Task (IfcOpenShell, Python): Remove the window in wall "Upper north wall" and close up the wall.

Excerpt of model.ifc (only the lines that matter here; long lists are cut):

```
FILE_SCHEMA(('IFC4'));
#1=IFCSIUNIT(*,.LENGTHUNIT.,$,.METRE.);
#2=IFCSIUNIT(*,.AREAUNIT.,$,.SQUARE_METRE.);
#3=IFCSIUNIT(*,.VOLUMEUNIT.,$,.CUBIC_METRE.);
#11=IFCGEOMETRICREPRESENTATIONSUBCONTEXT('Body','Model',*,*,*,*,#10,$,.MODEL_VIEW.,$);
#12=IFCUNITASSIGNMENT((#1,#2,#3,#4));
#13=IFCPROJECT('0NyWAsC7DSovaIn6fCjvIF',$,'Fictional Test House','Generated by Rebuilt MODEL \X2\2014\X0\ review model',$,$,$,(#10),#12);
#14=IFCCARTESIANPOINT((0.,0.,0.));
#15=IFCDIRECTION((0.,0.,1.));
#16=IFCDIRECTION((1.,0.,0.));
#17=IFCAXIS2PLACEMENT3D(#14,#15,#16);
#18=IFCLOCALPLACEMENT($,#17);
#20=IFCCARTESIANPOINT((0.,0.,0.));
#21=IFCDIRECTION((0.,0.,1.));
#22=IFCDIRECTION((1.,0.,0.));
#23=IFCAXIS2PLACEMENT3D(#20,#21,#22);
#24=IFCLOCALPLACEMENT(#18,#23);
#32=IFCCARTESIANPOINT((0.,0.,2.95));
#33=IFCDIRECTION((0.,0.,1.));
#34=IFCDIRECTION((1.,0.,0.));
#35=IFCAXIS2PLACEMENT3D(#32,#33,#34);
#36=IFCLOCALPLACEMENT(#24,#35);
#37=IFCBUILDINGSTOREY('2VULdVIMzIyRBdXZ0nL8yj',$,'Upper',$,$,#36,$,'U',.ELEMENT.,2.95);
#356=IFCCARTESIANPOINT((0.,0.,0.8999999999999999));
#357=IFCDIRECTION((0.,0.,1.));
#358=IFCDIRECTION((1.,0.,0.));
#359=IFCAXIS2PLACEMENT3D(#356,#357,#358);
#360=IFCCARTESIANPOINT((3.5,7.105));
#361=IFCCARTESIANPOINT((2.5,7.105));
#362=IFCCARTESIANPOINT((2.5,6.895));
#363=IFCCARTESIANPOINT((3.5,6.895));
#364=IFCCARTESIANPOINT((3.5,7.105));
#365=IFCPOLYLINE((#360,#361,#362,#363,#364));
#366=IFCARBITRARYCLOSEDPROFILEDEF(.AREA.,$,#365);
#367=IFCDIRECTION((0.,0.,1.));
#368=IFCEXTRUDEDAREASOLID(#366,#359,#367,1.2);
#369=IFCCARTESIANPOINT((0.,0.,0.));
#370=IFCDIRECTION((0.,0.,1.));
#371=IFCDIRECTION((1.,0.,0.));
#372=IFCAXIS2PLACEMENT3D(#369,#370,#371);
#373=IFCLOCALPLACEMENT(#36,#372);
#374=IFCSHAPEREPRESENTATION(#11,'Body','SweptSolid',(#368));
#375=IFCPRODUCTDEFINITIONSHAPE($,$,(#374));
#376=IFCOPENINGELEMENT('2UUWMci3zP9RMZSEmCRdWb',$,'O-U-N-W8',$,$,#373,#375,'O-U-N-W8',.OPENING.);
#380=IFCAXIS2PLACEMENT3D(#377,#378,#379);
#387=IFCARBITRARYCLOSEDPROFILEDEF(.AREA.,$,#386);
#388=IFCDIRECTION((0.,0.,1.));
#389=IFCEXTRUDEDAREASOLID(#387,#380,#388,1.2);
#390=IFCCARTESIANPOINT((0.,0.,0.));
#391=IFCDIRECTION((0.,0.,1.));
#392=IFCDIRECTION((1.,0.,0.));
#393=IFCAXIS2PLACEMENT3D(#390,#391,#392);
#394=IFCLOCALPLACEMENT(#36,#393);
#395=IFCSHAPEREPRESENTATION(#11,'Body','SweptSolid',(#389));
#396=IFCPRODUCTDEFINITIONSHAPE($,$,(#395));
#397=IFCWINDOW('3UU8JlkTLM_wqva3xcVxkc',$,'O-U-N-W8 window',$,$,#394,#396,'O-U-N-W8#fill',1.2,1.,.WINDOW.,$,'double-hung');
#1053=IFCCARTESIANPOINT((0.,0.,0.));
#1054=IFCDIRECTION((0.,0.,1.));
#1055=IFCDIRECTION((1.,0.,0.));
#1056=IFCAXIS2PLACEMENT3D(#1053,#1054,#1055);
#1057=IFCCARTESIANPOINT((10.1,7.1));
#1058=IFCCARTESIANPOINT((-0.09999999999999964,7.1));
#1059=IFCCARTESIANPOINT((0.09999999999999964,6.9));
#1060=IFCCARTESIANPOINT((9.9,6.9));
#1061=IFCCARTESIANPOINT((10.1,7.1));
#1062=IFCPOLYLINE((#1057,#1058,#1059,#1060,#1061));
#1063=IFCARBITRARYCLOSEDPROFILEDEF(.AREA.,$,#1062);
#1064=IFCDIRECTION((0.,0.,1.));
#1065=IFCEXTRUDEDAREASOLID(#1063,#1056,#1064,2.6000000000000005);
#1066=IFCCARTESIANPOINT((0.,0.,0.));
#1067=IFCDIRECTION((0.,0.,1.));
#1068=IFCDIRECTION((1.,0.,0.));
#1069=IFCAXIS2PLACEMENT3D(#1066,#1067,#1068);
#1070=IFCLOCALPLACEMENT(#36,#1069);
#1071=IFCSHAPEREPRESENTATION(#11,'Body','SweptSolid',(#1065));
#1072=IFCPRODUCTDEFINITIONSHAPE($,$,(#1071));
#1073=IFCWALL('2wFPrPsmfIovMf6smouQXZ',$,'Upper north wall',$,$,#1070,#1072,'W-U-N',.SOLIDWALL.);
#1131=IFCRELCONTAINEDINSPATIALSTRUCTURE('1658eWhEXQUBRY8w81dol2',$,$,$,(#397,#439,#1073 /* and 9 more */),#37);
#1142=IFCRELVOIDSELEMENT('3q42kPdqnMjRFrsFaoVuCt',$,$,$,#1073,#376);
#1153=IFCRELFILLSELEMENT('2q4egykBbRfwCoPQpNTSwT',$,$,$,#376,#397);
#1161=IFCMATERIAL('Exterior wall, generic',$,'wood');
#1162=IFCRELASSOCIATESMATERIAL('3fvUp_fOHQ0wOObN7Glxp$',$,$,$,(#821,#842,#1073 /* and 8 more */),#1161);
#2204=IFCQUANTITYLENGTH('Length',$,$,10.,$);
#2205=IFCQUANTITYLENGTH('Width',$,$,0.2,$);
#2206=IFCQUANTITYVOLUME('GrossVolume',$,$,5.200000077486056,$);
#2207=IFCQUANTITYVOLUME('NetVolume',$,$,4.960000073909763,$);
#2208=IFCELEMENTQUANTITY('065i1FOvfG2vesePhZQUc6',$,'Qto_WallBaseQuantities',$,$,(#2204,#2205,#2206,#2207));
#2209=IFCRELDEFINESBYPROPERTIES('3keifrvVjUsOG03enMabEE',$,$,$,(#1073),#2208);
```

```python
import ifcopenshell
import ifcopenshell.api.feature
import ifcopenshell.api.pset
import ifcopenshell.api.root
import ifcopenshell.geom
import ifcopenshell.util.element
import ifcopenshell.util.shape
import ifcopenshell.util.unit

model = ifcopenshell.open("model.ifc")
volume_scale = ifcopenshell.util.unit.calculate_unit_scale(model, "VOLUMEUNIT")
settings = ifcopenshell.geom.settings()


def volume(element):
    """Net volume in cubic metres, openings subtracted."""
    shape = ifcopenshell.geom.create_shape(settings, element)
    return ifcopenshell.util.shape.get_volume(shape.geometry)


window = model.by_guid("3UU8JlkTLM_wqva3xcVxkc")
opening = window.FillsVoids[0].RelatingOpeningElement
wall = opening.VoidsElements[0].RelatingBuildingElement
before = volume(wall)

ifcopenshell.api.root.remove_product(model, product=window)
ifcopenshell.api.feature.remove_feature(model, feature=opening)

after = volume(wall)

# Update the wall's stored quantities.
qto = model.by_id(ifcopenshell.util.element.get_pset(wall, "Qto_WallBaseQuantities", should_inherit=False)["id"])
ifcopenshell.api.pset.edit_qto(model, qto=qto, properties={"NetVolume": after / volume_scale})

print(f"wall volume {before:.3f} -> {after:.3f} m3")

model.write("model_edited.ifc")
```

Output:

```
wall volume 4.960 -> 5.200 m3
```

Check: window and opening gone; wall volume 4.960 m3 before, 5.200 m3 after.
